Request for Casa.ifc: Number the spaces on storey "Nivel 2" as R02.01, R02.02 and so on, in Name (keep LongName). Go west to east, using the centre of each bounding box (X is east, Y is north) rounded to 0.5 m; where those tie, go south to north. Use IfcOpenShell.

First a look at what the model holds.

```python
import ifcopenshell
import ifcopenshell.util.element
import ifcopenshell.util.placement

model = ifcopenshell.open("Casa.ifc")
print(model.schema)
storey = next(s for s in model.by_type("IfcBuildingStorey") if s.Name == "Nivel 2")
spaces = [e for e in ifcopenshell.util.element.get_decomposition(storey) if e.is_a("IfcSpace")]
for e in sorted(spaces, key=lambda e: e.id()):
    origin = ifcopenshell.util.placement.get_local_placement(e.ObjectPlacement)[:3, 3]
    print(e.id(), e.Name, e.LongName, origin.round(2) + 0.0, sep=" | ")
```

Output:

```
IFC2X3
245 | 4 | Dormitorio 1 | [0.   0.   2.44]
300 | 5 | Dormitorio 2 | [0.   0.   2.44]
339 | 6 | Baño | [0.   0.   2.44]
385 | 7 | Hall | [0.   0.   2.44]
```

```python
import ifcopenshell
import ifcopenshell.geom
import ifcopenshell.util.element
import ifcopenshell.util.shape

model = ifcopenshell.open("Casa.ifc")
settings = ifcopenshell.geom.settings()
settings.set("use-world-coords", True)


def centre(element):
    shape = ifcopenshell.geom.create_shape(settings, element)
    return ifcopenshell.util.shape.get_bbox_centroid(shape.geometry)


storey = next(s for s in model.by_type("IfcBuildingStorey") if s.Name == "Nivel 2")
spaces = [e for e in ifcopenshell.util.element.get_decomposition(storey) if e.is_a("IfcSpace")]

# Insertion points can sit at a corner or the storey origin, so sort by the geometry (in metres).
centres = {e: centre(e) for e in spaces}
spaces.sort(key=lambda e: (round(centres[e][0] / 0.5), centres[e][1]))

for i, e in enumerate(spaces, start=1):
    number = f"R02.{i:02d}"
    e.Name = number
    print(e.id(), number)

model.write("Casa-out.ifc")
```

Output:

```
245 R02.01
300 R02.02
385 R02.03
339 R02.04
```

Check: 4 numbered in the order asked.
